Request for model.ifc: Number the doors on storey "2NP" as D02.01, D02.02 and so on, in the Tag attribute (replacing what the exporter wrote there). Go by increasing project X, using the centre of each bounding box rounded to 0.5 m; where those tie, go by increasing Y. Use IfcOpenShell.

First a look at what the model holds.

```python
import ifcopenshell
import ifcopenshell.util.element
import ifcopenshell.util.placement

model = ifcopenshell.open("model.ifc")
print(model.schema)
storey = next(s for s in model.by_type("IfcBuildingStorey") if s.Name == "2NP")
doors = [e for e in ifcopenshell.util.element.get_decomposition(storey) if e.is_a("IfcDoor")]
for e in sorted(doors, key=lambda e: e.id()):
    origin = ifcopenshell.util.placement.get_local_placement(e.ObjectPlacement)[:3, 3]
    print(e.id(), e.Tag, e.Name, origin.round(2) + 0.0, sep=" | ")
```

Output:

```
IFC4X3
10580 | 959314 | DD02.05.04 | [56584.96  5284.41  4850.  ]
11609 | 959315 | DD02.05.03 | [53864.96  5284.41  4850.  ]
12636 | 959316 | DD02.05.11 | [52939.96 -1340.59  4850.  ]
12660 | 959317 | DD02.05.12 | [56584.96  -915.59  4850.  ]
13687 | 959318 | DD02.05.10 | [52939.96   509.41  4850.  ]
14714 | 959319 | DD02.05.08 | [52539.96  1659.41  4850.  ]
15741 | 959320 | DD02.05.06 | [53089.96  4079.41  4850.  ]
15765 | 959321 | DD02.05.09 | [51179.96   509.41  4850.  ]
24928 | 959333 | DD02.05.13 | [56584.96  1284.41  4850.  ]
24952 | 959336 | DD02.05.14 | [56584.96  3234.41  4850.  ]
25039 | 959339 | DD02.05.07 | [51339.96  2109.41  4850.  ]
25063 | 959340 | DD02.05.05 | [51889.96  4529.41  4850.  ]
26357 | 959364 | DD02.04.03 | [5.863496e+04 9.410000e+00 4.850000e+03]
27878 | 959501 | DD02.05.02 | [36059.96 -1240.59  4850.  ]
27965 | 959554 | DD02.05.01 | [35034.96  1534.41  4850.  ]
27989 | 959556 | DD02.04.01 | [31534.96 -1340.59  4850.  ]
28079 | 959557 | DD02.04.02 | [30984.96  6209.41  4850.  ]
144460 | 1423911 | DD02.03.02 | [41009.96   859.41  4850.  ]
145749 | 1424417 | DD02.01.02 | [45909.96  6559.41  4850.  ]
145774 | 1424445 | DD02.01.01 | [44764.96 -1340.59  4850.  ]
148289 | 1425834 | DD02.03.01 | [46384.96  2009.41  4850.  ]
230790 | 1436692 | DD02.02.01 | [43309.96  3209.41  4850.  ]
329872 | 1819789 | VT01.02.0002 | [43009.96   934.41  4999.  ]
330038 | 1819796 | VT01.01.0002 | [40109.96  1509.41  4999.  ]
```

```python
import ifcopenshell
import ifcopenshell.geom
import ifcopenshell.util.element
import ifcopenshell.util.shape

model = ifcopenshell.open("model.ifc")
settings = ifcopenshell.geom.settings()
settings.set("use-world-coords", True)


def centre(element):
    shape = ifcopenshell.geom.create_shape(settings, element)
    return ifcopenshell.util.shape.get_bbox_centroid(shape.geometry)


storey = next(s for s in model.by_type("IfcBuildingStorey") if s.Name == "2NP")
doors = [e for e in ifcopenshell.util.element.get_decomposition(storey) if e.is_a("IfcDoor")]

# Insertion points can sit at a corner or the storey origin, so sort by the geometry (in metres).
centres = {e: centre(e) for e in doors}
doors.sort(key=lambda e: (round(centres[e][0] / 0.5), centres[e][1]))

for i, e in enumerate(doors, start=1):
    number = f"D02.{i:02d}"
    e.Tag = number
    print(e.id(), number)

model.write("model_updated.ifc")
```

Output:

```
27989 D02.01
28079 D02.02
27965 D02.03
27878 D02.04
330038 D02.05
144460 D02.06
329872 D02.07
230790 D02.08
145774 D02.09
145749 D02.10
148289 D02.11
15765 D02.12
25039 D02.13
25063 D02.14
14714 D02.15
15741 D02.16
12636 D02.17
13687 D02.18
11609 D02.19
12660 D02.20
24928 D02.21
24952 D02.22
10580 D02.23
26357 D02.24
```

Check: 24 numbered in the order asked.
